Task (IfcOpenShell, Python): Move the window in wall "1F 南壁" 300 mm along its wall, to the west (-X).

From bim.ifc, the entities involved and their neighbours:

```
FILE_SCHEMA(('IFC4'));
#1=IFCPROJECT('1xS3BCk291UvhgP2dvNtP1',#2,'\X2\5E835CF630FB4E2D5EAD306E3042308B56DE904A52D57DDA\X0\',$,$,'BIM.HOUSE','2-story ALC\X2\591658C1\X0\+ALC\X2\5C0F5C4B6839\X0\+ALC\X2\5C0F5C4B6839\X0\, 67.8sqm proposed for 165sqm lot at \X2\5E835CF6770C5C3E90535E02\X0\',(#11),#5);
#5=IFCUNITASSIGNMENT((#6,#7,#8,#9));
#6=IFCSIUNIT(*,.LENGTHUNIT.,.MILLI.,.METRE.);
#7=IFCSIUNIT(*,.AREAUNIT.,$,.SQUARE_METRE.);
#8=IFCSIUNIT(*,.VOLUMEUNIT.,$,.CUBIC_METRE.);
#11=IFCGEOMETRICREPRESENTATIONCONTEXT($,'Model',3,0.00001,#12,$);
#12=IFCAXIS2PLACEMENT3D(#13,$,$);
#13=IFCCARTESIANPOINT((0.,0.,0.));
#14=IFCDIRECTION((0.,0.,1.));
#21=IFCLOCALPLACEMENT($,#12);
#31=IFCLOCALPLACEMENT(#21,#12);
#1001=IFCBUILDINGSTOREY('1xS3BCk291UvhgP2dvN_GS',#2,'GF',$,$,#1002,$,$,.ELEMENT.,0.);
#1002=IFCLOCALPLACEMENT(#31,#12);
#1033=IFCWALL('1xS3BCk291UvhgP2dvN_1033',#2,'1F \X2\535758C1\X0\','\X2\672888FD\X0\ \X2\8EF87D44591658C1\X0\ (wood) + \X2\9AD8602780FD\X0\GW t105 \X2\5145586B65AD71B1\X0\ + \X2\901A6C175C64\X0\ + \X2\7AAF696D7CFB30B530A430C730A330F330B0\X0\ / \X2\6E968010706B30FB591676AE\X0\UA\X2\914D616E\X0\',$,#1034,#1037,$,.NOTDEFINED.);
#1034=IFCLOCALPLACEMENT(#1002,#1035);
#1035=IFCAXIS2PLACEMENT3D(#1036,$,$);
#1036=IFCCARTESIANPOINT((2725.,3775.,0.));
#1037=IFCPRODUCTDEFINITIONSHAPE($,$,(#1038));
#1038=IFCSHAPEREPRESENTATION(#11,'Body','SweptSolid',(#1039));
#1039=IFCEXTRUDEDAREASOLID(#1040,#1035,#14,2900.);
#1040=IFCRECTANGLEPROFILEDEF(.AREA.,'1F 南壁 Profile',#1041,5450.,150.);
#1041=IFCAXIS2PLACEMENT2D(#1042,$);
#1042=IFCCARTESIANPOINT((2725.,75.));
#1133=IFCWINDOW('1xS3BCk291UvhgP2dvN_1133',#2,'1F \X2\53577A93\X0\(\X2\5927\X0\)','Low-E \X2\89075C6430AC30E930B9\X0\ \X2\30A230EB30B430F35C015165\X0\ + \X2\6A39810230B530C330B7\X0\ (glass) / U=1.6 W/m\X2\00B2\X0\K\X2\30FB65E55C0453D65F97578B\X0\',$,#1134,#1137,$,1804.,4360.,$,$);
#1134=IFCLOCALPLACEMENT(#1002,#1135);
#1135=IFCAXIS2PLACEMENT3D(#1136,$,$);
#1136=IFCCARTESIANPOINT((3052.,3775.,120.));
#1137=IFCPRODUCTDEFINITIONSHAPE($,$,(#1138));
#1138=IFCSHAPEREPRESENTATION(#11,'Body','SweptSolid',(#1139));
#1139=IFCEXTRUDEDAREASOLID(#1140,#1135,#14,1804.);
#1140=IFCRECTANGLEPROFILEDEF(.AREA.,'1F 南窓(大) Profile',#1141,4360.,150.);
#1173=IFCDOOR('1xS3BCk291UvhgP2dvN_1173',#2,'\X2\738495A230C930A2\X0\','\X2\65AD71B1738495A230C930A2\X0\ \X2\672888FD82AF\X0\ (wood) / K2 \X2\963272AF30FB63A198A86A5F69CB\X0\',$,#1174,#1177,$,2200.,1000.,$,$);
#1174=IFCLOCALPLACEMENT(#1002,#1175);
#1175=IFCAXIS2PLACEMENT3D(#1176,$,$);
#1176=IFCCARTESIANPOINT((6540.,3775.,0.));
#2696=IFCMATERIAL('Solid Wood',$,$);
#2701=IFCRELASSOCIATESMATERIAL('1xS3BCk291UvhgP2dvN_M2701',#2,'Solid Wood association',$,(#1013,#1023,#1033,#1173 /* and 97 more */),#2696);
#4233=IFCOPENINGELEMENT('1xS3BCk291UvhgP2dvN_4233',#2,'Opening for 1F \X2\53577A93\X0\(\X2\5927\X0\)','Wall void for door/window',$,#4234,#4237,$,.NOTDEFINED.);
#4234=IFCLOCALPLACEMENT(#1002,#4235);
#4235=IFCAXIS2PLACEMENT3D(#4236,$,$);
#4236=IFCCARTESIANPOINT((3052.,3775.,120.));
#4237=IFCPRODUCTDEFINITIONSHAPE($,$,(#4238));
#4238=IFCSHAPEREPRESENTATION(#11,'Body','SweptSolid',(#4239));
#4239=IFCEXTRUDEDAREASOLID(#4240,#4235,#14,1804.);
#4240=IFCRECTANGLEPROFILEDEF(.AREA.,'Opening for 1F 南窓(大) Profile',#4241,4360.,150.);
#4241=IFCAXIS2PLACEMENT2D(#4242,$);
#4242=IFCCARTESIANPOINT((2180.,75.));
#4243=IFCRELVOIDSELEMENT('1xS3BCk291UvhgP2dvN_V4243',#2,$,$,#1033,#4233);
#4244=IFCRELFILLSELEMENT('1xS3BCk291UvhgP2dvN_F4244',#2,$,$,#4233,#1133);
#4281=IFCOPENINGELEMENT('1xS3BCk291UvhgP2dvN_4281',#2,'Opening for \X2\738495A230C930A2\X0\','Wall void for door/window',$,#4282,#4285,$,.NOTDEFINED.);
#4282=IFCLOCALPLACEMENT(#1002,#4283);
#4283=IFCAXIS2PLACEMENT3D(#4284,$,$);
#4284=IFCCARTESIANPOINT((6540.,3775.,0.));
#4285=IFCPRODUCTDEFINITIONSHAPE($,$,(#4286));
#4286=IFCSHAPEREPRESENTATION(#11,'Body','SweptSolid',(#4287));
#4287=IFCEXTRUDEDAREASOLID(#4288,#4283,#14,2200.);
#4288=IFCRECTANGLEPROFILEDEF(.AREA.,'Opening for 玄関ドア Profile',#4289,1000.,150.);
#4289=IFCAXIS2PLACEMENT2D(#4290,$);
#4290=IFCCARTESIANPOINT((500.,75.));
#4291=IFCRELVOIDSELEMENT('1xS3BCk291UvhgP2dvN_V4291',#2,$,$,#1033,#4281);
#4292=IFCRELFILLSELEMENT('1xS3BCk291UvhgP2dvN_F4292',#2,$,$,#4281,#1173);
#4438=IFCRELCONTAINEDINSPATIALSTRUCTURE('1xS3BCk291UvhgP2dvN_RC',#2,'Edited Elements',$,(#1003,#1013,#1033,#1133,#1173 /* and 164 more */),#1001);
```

```python
import ifcopenshell
import ifcopenshell.api.geometry
import ifcopenshell.util.placement
import ifcopenshell.util.unit

model = ifcopenshell.open("bim.ifc")
unit_scale = ifcopenshell.util.unit.calculate_unit_scale(model)

window = model.by_guid("1xS3BCk291UvhgP2dvN_1133")
opening = window.FillsVoids[0].RelatingOpeningElement
wall = opening.VoidsElements[0].RelatingBuildingElement

wall_matrix = ifcopenshell.util.placement.get_local_placement(wall.ObjectPlacement)
shift = wall_matrix[:3, 0] * -0.3 / unit_scale
before = ifcopenshell.util.placement.get_local_placement(window.ObjectPlacement)[:3, 3].copy()

# The window is not placed relative to its opening, so move both.
for product in (opening, window):
    matrix = ifcopenshell.util.placement.get_local_placement(product.ObjectPlacement)
    matrix[:3, 3] += shift
    ifcopenshell.api.geometry.edit_object_placement(model, product=product, matrix=matrix, is_si=False)

after = ifcopenshell.util.placement.get_local_placement(window.ObjectPlacement)[:3, 3]
print("window moved by", (after - before).round(3) + 0.0)

model.write("bim_updated.ifc")
```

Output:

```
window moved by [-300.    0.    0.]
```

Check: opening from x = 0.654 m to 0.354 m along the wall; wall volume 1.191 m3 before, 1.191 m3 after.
